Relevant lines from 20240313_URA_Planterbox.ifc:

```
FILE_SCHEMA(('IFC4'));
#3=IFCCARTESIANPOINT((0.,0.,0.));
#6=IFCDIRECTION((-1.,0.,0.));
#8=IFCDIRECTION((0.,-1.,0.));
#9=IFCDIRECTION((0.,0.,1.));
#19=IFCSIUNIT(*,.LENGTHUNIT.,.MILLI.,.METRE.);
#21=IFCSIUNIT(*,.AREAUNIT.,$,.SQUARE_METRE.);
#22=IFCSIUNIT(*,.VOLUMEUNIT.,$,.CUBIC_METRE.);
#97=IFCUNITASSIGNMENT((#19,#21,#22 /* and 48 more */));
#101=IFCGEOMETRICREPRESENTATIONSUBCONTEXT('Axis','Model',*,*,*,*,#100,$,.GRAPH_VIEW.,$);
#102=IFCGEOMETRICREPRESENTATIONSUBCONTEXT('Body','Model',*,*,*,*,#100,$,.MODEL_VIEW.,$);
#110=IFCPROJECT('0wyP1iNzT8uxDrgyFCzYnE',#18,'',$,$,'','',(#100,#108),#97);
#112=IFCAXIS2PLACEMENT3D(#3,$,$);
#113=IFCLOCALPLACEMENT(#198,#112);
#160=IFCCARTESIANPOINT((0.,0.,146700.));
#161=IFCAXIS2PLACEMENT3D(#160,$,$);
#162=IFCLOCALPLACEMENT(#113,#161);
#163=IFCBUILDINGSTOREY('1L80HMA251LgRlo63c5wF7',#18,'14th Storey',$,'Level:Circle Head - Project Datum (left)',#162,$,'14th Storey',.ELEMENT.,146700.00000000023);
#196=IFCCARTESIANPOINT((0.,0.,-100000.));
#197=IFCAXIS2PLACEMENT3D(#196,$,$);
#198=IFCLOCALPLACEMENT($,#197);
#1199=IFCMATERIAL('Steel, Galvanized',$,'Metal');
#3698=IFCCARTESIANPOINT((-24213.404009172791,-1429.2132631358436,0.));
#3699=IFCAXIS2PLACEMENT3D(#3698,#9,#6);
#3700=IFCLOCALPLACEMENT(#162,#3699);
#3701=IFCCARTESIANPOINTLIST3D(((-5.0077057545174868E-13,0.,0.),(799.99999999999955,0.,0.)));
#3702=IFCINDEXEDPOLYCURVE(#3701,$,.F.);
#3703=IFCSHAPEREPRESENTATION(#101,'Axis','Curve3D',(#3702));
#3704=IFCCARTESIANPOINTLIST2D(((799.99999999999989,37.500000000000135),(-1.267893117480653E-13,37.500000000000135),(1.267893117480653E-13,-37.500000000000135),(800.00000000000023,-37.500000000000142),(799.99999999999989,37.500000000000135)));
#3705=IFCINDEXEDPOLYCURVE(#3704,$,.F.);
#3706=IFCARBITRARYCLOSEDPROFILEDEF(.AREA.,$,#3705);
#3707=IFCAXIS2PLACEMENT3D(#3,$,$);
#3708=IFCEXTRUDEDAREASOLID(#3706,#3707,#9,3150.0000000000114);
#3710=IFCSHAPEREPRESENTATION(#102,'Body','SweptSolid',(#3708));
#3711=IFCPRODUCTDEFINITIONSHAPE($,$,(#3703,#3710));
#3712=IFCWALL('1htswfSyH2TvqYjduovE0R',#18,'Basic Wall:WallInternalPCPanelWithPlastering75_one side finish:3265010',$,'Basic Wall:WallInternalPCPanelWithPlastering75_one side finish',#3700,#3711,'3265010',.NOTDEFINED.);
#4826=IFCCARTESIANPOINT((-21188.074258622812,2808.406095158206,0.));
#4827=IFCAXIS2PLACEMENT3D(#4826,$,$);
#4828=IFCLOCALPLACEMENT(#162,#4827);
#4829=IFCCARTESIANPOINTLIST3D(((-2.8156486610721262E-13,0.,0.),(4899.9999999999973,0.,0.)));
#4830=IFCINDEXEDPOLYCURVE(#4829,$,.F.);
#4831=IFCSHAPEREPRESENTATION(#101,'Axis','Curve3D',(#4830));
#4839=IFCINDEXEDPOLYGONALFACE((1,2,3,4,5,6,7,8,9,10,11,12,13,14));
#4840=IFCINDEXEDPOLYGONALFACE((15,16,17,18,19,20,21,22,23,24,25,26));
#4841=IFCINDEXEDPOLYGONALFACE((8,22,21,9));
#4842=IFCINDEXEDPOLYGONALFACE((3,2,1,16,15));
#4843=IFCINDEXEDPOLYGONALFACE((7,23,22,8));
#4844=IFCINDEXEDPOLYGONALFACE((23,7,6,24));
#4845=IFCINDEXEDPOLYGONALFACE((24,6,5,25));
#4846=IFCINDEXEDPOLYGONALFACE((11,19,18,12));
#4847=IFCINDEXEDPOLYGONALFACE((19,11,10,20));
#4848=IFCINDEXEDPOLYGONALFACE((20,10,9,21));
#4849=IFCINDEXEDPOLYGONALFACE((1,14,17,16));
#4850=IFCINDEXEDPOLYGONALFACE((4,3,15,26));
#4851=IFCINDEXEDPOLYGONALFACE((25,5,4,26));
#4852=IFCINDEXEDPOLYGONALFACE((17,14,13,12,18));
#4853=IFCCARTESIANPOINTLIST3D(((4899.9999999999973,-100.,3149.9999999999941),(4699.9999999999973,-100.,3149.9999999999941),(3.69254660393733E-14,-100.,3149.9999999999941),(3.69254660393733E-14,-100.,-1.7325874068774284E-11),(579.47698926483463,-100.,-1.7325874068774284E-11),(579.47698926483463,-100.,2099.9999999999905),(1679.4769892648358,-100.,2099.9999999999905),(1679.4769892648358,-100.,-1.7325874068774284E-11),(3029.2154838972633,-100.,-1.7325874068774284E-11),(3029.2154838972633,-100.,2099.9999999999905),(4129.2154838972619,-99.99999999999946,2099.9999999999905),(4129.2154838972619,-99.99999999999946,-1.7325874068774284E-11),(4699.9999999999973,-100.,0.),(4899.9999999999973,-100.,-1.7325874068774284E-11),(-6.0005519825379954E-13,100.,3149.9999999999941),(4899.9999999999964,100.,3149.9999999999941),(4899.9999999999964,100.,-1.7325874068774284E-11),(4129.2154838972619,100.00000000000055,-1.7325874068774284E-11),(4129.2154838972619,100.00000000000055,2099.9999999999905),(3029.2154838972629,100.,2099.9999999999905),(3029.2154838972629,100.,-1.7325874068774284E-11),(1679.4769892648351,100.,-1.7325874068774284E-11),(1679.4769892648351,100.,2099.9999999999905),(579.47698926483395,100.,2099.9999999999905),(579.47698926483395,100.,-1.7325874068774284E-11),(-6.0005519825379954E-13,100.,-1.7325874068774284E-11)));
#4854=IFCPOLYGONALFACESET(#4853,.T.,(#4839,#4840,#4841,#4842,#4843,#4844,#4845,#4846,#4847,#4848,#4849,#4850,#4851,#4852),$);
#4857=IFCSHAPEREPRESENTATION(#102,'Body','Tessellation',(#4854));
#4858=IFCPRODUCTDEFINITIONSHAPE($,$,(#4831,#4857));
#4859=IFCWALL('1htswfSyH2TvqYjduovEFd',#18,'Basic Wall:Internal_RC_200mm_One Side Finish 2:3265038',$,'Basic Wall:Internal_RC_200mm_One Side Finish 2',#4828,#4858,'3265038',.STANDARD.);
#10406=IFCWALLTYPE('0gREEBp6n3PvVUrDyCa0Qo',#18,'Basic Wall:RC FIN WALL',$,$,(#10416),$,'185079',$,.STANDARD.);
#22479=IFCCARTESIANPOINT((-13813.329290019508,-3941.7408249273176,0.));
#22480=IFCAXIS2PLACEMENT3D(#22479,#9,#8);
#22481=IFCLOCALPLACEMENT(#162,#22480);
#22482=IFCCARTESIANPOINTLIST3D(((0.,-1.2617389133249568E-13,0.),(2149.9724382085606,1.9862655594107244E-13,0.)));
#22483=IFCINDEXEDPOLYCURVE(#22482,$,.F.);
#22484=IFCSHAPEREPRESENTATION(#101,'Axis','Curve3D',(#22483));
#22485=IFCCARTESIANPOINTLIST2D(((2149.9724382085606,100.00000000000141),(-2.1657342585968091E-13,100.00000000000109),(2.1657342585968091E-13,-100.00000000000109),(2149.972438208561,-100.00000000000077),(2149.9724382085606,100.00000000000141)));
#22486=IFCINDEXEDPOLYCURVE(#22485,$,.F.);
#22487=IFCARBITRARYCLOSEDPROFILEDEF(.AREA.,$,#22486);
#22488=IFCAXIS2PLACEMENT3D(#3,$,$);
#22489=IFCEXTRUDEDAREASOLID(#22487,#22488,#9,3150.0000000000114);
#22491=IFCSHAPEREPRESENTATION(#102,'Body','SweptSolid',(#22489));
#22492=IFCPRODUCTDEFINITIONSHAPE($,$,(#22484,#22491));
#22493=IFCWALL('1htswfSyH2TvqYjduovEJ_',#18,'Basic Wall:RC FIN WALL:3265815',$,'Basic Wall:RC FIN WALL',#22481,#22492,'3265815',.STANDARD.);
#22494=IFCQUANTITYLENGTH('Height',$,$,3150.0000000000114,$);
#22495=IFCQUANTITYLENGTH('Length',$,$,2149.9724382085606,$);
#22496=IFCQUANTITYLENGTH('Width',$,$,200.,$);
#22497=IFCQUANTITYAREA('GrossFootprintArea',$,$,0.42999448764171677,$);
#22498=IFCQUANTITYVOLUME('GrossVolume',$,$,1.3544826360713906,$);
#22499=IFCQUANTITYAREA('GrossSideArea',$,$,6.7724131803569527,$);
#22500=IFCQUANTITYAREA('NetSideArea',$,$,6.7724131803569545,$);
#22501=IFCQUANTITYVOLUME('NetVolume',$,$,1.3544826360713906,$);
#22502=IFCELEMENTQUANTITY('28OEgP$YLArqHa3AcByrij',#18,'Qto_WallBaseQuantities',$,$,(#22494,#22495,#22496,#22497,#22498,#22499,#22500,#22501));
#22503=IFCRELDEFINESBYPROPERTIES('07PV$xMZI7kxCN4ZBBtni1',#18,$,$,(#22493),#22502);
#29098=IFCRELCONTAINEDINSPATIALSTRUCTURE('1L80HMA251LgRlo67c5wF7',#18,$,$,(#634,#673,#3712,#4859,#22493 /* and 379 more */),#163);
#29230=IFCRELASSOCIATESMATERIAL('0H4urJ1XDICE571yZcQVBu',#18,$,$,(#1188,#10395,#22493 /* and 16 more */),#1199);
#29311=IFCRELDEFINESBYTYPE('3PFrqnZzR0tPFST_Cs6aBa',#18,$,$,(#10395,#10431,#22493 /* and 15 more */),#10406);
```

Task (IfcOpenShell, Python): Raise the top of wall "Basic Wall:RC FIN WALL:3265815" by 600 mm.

```python
import ifcopenshell
import ifcopenshell.api.pset
import ifcopenshell.geom
import ifcopenshell.util.element
import ifcopenshell.util.representation
import ifcopenshell.util.shape
import ifcopenshell.util.unit

model = ifcopenshell.open("20240313_URA_Planterbox.ifc")
unit_scale = ifcopenshell.util.unit.calculate_unit_scale(model)
area_scale = ifcopenshell.util.unit.calculate_unit_scale(model, "AREAUNIT")
volume_scale = ifcopenshell.util.unit.calculate_unit_scale(model, "VOLUMEUNIT")
settings = ifcopenshell.geom.settings()


def volume(element):
    """Net volume in cubic metres, openings subtracted."""
    shape = ifcopenshell.geom.create_shape(settings, element)
    return ifcopenshell.util.shape.get_volume(shape.geometry)


wall = model.by_guid("1htswfSyH2TvqYjduovEJ_")
before = volume(wall)

body = ifcopenshell.util.representation.get_representation(wall, "Model", "Body")
solid = body.Items[0]
old_height = solid.Depth
solid.Depth += 600.0
after = volume(wall)
thickness = 0.2  # wall thickness in metres

# Update the stored height, areas and volumes.
qto = model.by_id(ifcopenshell.util.element.get_pset(wall, "Qto_WallBaseQuantities", should_inherit=False)["id"])
ifcopenshell.api.pset.edit_qto(model, qto=qto, properties={
    "Height": solid.Depth,
    "GrossVolume": ifcopenshell.util.element.get_pset(wall, "Qto_WallBaseQuantities", "GrossVolume") * solid.Depth / old_height,
    "GrossSideArea": ifcopenshell.util.element.get_pset(wall, "Qto_WallBaseQuantities", "GrossSideArea") * solid.Depth / old_height,
    "NetSideArea": after / thickness / area_scale,
    "NetVolume": after / volume_scale,
})

print(f"height {old_height:g} -> {solid.Depth:g}, volume {before:.3f} -> {after:.3f} m3")

model.write("20240313_URA_Planterbox_updated.ifc")
```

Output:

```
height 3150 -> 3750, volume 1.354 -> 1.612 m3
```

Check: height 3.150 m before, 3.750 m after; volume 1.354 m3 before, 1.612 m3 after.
